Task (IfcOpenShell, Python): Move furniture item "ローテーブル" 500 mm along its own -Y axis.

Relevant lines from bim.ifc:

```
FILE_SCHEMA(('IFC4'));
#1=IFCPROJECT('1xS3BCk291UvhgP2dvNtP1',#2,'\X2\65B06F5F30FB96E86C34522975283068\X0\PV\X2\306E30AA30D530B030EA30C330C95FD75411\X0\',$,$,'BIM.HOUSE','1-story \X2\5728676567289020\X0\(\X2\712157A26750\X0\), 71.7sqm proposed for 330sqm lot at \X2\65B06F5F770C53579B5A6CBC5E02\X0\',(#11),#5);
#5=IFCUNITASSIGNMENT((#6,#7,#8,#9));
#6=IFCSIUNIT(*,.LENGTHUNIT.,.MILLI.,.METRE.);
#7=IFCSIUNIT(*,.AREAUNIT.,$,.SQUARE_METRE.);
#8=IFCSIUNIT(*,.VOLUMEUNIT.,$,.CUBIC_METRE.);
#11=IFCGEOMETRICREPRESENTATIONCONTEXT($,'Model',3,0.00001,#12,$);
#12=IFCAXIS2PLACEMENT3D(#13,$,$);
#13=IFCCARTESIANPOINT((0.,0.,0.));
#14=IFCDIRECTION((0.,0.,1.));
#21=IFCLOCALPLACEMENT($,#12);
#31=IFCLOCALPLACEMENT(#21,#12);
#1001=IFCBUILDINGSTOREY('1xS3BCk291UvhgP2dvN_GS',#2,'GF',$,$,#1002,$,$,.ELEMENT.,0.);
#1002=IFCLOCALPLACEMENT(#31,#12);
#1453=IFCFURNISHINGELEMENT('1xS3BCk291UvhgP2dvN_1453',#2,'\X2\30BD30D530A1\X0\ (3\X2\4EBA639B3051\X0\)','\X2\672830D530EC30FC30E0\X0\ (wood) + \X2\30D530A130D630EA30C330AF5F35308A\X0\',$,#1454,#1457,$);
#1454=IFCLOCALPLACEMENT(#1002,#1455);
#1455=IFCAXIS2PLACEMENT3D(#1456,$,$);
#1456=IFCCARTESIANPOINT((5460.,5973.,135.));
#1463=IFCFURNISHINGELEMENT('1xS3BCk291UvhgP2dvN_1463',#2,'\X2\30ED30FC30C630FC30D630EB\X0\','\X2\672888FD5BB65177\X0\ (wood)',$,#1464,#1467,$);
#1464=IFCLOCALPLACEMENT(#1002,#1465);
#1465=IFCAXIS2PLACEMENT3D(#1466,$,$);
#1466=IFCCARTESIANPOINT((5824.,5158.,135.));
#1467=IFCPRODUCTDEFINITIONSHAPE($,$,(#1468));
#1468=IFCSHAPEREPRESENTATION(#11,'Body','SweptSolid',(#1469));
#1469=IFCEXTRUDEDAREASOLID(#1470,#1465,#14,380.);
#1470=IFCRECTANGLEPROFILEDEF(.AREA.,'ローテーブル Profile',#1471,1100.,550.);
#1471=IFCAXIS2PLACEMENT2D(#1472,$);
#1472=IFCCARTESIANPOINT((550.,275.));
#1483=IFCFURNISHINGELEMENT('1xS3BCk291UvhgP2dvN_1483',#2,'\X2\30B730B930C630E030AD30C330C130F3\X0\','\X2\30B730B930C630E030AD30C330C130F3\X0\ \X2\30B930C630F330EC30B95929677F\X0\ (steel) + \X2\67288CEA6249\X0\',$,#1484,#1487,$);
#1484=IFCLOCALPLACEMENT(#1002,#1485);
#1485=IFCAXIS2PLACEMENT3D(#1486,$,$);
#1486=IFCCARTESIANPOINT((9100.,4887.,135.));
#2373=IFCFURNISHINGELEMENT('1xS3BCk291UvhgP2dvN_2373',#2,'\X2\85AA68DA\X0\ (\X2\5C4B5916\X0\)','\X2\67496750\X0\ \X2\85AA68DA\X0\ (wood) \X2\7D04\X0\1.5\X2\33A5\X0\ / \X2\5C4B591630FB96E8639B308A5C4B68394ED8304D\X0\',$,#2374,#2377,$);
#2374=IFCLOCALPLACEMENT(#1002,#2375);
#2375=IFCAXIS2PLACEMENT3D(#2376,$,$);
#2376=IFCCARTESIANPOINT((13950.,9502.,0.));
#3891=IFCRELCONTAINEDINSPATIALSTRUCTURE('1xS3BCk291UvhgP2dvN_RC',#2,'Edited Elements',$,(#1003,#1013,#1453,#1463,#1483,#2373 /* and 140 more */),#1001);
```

```python
import ifcopenshell
import ifcopenshell.api.geometry
import ifcopenshell.util.placement
import ifcopenshell.util.unit

model = ifcopenshell.open("bim.ifc")
unit_scale = ifcopenshell.util.unit.calculate_unit_scale(model)

item = model.by_guid("1xS3BCk291UvhgP2dvN_1463")
matrix = ifcopenshell.util.placement.get_local_placement(item.ObjectPlacement)
matrix[:3, 3] -= matrix[:3, 1] * 0.5 / unit_scale
ifcopenshell.api.geometry.edit_object_placement(model, product=item, matrix=matrix, is_si=False)

print(ifcopenshell.util.placement.get_local_placement(item.ObjectPlacement).round(3) + 0.0)

model.write("bim-out.ifc")
```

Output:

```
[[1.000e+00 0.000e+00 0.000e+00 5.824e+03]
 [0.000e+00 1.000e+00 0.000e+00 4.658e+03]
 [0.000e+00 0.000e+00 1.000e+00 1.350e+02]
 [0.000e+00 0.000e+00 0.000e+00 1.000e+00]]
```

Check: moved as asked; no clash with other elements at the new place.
